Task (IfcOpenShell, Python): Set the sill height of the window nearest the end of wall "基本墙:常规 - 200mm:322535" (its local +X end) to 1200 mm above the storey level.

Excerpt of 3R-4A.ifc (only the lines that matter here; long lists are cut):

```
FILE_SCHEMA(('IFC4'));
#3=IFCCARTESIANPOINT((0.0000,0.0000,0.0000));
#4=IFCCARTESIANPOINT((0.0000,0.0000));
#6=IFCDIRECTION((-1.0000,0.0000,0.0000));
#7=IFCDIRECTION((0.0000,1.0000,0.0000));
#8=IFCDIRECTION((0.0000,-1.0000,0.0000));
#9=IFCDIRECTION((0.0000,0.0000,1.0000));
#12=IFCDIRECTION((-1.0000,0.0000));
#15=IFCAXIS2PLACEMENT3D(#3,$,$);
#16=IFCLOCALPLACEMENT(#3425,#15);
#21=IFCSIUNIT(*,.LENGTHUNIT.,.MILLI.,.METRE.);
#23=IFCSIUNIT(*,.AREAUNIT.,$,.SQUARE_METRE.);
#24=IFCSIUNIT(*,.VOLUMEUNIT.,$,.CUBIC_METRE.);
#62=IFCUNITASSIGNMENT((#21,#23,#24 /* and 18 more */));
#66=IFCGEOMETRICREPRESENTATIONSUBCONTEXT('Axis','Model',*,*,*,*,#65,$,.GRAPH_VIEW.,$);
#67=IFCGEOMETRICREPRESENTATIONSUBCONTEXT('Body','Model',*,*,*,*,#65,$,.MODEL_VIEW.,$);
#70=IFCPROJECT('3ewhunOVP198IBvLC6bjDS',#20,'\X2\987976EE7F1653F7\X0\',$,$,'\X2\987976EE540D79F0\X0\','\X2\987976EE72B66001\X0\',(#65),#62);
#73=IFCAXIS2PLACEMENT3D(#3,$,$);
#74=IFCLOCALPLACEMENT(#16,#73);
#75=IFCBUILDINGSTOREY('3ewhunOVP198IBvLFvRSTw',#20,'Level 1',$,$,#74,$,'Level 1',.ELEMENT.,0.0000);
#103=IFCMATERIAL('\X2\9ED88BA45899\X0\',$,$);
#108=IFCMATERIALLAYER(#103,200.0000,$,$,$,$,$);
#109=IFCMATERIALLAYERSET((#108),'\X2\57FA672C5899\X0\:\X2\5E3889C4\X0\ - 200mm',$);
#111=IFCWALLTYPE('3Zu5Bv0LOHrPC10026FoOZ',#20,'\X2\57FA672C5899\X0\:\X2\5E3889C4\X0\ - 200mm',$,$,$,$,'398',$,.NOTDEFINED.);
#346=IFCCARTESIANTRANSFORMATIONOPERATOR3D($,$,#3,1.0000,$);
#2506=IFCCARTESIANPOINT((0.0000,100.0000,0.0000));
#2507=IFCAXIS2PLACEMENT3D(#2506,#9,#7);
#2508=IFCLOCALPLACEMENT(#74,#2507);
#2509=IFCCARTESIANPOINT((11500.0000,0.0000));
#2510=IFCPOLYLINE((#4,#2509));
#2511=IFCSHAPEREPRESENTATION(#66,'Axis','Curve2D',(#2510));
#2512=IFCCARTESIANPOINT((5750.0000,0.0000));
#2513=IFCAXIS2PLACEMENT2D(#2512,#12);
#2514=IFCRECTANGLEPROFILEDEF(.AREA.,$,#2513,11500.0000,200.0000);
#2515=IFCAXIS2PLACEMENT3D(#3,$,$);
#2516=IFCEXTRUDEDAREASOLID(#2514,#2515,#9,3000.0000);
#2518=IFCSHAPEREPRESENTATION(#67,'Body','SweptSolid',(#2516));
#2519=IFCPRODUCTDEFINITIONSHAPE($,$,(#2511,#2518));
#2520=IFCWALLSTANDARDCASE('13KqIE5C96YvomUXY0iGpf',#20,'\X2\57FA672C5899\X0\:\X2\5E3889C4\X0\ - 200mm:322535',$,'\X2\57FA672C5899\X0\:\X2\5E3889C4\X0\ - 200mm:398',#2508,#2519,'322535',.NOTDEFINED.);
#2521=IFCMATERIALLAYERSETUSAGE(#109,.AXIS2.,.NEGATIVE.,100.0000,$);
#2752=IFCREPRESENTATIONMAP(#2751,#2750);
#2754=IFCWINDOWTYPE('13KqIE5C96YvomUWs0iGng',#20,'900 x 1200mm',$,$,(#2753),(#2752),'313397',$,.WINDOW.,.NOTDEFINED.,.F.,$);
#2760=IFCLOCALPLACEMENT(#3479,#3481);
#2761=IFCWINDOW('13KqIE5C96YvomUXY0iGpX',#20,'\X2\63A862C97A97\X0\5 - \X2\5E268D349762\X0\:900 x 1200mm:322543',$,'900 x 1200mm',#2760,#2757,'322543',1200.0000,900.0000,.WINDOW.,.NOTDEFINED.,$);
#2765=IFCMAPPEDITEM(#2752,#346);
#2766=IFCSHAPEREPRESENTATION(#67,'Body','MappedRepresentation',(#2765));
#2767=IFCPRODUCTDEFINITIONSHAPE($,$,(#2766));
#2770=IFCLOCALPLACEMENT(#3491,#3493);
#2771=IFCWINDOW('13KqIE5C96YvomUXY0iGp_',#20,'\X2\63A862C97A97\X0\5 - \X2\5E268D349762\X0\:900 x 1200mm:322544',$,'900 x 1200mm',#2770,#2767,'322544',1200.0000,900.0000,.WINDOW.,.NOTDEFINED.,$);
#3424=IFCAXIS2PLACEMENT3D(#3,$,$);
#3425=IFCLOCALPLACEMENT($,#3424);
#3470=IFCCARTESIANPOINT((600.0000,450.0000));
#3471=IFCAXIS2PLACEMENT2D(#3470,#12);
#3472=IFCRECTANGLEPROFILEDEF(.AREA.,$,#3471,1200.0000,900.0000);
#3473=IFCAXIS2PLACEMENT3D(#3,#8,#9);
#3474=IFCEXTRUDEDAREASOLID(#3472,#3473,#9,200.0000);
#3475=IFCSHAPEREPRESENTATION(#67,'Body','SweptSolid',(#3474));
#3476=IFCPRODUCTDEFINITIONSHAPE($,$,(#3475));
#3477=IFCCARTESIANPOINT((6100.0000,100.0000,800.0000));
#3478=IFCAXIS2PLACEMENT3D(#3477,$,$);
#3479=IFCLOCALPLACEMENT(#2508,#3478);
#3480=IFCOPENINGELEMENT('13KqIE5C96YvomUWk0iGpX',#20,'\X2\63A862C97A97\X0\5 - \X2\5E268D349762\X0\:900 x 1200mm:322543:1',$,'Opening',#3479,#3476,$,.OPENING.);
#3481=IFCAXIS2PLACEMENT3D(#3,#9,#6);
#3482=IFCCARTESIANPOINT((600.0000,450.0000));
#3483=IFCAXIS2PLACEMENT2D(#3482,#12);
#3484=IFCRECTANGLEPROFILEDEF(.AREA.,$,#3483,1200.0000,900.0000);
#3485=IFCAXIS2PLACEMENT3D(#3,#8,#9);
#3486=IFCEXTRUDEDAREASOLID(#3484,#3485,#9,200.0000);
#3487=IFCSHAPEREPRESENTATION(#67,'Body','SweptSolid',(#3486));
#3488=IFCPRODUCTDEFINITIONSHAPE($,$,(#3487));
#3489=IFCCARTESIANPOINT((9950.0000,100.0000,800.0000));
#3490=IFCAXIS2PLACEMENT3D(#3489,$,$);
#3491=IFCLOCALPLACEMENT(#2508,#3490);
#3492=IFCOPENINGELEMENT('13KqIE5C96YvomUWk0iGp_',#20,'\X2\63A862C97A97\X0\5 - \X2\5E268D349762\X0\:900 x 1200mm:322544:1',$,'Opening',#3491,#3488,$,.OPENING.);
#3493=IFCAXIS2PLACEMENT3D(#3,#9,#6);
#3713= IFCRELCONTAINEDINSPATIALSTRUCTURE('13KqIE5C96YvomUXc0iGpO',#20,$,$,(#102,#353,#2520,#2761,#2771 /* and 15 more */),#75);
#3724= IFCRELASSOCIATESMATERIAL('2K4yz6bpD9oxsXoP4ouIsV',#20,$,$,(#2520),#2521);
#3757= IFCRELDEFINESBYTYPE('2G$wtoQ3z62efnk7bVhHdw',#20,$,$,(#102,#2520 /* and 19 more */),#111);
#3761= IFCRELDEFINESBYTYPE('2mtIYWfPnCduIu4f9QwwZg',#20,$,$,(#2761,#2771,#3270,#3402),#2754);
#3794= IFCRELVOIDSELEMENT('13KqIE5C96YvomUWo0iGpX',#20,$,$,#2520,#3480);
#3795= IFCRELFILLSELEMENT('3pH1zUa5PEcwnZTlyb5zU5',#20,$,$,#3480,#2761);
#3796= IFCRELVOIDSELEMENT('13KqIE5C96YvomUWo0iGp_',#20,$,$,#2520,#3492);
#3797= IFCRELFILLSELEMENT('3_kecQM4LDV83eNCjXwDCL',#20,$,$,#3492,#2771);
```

```python
import numpy as np
import ifcopenshell
import ifcopenshell.api.geometry
import ifcopenshell.geom
import ifcopenshell.util.element
import ifcopenshell.util.placement
import ifcopenshell.util.shape
import ifcopenshell.util.unit

model = ifcopenshell.open("3R-4A.ifc")
unit_scale = ifcopenshell.util.unit.calculate_unit_scale(model)

window = model.by_id(2771)
opening = window.FillsVoids[0].RelatingOpeningElement
storey = ifcopenshell.util.element.get_container(window, ifc_class="IfcBuildingStorey")
level = ifcopenshell.util.placement.get_local_placement(storey.ObjectPlacement)[2, 3]

# The opening's origin need not be at the sill, so measure its lowest point.
shape = ifcopenshell.geom.create_shape(ifcopenshell.geom.settings(), opening)
bottom = ifcopenshell.util.shape.get_shape_bottom_elevation(shape, shape.geometry) / unit_scale
dz = level + 1.2 / unit_scale - bottom

shift = np.array([0.0, 0.0, dz])
# The window is placed relative to its opening, so it follows when the opening moves.
matrix = ifcopenshell.util.placement.get_local_placement(opening.ObjectPlacement)
matrix[:3, 3] += shift
ifcopenshell.api.geometry.edit_object_placement(
    model, product=opening, matrix=matrix, is_si=False, should_transform_children=True
)

print(f"moved by {dz * unit_scale:+.3f} m")

model.write("3R-4A_updated.ifc")
```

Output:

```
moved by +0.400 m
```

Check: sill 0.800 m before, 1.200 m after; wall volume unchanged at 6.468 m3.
